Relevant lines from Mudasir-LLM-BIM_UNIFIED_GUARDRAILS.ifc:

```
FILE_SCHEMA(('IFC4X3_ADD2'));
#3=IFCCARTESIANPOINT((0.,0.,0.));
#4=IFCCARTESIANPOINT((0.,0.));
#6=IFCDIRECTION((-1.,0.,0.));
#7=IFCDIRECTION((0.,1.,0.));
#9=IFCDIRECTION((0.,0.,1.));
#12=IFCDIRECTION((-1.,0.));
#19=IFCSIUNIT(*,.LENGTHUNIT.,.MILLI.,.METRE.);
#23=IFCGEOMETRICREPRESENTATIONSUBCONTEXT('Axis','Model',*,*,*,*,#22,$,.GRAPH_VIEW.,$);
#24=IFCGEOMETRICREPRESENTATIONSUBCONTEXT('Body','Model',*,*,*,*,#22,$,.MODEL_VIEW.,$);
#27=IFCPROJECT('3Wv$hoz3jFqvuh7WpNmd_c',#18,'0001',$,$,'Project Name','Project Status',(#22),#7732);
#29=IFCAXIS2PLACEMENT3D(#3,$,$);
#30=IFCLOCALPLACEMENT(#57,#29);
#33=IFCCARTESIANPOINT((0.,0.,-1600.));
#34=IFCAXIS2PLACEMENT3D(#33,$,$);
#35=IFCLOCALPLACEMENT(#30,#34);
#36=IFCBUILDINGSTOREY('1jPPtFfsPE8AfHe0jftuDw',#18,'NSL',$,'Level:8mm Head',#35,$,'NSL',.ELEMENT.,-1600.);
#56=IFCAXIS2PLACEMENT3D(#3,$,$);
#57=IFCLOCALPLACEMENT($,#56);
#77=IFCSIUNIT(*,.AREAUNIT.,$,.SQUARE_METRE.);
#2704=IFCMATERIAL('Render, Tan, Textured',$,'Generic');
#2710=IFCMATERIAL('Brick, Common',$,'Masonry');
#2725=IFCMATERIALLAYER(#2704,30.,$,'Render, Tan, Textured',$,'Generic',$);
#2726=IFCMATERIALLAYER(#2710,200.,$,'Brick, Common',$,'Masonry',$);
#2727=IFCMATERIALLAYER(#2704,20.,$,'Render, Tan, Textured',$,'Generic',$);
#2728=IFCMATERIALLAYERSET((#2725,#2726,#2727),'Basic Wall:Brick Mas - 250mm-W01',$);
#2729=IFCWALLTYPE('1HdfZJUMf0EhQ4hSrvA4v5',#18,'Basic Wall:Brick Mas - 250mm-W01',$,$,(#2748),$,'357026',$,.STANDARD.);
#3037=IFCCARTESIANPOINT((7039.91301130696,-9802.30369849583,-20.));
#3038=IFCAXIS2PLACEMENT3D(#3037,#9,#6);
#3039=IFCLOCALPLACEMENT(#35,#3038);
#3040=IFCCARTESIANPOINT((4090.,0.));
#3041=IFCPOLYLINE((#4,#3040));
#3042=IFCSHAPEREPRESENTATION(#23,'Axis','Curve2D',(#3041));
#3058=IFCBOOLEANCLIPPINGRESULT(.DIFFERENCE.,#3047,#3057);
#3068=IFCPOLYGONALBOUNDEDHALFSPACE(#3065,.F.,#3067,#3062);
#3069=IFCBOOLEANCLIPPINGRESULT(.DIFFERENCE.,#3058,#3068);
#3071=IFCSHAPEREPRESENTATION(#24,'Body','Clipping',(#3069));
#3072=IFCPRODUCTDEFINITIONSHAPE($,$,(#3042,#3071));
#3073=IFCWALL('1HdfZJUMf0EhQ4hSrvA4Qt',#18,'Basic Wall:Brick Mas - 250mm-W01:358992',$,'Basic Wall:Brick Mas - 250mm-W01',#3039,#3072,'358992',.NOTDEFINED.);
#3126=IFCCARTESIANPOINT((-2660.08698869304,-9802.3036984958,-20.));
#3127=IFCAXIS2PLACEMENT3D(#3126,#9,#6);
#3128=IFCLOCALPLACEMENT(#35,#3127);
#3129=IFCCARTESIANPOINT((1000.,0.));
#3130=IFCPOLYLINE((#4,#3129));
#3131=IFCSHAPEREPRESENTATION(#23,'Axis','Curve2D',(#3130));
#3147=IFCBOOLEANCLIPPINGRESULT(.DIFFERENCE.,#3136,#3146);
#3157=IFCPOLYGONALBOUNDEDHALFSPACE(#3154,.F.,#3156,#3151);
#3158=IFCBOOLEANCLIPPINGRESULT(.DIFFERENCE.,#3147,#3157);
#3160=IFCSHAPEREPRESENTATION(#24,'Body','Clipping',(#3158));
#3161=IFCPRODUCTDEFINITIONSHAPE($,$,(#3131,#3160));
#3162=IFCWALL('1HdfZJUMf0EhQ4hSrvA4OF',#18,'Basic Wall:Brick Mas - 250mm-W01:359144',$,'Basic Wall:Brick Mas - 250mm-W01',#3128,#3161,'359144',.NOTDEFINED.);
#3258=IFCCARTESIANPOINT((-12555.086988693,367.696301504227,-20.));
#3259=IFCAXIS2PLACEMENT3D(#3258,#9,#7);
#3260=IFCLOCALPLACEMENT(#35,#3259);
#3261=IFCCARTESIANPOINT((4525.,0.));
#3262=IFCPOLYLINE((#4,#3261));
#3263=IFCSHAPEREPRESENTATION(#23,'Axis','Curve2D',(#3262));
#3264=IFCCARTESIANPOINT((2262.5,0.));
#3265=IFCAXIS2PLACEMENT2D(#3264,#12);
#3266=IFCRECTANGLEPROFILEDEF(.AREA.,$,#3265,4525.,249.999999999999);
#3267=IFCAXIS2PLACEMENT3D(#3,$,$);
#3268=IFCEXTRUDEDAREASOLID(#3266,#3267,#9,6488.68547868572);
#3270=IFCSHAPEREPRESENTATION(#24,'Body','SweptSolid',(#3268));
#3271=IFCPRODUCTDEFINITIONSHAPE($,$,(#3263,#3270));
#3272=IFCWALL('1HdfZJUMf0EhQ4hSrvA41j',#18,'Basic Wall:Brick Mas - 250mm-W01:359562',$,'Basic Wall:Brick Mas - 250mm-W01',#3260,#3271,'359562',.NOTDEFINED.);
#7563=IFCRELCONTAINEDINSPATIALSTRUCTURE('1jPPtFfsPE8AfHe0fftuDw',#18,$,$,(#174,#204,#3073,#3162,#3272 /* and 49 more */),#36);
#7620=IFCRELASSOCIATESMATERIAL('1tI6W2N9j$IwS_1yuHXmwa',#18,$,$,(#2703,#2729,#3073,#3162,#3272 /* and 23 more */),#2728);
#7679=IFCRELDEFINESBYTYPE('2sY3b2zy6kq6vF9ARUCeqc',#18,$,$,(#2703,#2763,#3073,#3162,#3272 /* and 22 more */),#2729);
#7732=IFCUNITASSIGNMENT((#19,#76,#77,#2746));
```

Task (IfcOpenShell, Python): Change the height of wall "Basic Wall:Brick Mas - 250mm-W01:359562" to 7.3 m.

```python
import ifcopenshell
import ifcopenshell.geom
import ifcopenshell.util.representation
import ifcopenshell.util.shape
import ifcopenshell.util.unit

model = ifcopenshell.open("Mudasir-LLM-BIM_UNIFIED_GUARDRAILS.ifc")
unit_scale = ifcopenshell.util.unit.calculate_unit_scale(model)
settings = ifcopenshell.geom.settings()


def volume(element):
    """Net volume in cubic metres, openings subtracted."""
    shape = ifcopenshell.geom.create_shape(settings, element)
    return ifcopenshell.util.shape.get_volume(shape.geometry)


wall = model.by_guid("1HdfZJUMf0EhQ4hSrvA41j")
before = volume(wall)

body = ifcopenshell.util.representation.get_representation(wall, "Model", "Body")
solid = body.Items[0]
old_height = solid.Depth
solid.Depth = 7.3 / unit_scale
after = volume(wall)

print(f"height {old_height:g} -> {solid.Depth:g}, volume {before:.3f} -> {after:.3f} m3")

model.write("Mudasir-LLM-BIM_UNIFIED_GUARDRAILS_updated.ifc")
```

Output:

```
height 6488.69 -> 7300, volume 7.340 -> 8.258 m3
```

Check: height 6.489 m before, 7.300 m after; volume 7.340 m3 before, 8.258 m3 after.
